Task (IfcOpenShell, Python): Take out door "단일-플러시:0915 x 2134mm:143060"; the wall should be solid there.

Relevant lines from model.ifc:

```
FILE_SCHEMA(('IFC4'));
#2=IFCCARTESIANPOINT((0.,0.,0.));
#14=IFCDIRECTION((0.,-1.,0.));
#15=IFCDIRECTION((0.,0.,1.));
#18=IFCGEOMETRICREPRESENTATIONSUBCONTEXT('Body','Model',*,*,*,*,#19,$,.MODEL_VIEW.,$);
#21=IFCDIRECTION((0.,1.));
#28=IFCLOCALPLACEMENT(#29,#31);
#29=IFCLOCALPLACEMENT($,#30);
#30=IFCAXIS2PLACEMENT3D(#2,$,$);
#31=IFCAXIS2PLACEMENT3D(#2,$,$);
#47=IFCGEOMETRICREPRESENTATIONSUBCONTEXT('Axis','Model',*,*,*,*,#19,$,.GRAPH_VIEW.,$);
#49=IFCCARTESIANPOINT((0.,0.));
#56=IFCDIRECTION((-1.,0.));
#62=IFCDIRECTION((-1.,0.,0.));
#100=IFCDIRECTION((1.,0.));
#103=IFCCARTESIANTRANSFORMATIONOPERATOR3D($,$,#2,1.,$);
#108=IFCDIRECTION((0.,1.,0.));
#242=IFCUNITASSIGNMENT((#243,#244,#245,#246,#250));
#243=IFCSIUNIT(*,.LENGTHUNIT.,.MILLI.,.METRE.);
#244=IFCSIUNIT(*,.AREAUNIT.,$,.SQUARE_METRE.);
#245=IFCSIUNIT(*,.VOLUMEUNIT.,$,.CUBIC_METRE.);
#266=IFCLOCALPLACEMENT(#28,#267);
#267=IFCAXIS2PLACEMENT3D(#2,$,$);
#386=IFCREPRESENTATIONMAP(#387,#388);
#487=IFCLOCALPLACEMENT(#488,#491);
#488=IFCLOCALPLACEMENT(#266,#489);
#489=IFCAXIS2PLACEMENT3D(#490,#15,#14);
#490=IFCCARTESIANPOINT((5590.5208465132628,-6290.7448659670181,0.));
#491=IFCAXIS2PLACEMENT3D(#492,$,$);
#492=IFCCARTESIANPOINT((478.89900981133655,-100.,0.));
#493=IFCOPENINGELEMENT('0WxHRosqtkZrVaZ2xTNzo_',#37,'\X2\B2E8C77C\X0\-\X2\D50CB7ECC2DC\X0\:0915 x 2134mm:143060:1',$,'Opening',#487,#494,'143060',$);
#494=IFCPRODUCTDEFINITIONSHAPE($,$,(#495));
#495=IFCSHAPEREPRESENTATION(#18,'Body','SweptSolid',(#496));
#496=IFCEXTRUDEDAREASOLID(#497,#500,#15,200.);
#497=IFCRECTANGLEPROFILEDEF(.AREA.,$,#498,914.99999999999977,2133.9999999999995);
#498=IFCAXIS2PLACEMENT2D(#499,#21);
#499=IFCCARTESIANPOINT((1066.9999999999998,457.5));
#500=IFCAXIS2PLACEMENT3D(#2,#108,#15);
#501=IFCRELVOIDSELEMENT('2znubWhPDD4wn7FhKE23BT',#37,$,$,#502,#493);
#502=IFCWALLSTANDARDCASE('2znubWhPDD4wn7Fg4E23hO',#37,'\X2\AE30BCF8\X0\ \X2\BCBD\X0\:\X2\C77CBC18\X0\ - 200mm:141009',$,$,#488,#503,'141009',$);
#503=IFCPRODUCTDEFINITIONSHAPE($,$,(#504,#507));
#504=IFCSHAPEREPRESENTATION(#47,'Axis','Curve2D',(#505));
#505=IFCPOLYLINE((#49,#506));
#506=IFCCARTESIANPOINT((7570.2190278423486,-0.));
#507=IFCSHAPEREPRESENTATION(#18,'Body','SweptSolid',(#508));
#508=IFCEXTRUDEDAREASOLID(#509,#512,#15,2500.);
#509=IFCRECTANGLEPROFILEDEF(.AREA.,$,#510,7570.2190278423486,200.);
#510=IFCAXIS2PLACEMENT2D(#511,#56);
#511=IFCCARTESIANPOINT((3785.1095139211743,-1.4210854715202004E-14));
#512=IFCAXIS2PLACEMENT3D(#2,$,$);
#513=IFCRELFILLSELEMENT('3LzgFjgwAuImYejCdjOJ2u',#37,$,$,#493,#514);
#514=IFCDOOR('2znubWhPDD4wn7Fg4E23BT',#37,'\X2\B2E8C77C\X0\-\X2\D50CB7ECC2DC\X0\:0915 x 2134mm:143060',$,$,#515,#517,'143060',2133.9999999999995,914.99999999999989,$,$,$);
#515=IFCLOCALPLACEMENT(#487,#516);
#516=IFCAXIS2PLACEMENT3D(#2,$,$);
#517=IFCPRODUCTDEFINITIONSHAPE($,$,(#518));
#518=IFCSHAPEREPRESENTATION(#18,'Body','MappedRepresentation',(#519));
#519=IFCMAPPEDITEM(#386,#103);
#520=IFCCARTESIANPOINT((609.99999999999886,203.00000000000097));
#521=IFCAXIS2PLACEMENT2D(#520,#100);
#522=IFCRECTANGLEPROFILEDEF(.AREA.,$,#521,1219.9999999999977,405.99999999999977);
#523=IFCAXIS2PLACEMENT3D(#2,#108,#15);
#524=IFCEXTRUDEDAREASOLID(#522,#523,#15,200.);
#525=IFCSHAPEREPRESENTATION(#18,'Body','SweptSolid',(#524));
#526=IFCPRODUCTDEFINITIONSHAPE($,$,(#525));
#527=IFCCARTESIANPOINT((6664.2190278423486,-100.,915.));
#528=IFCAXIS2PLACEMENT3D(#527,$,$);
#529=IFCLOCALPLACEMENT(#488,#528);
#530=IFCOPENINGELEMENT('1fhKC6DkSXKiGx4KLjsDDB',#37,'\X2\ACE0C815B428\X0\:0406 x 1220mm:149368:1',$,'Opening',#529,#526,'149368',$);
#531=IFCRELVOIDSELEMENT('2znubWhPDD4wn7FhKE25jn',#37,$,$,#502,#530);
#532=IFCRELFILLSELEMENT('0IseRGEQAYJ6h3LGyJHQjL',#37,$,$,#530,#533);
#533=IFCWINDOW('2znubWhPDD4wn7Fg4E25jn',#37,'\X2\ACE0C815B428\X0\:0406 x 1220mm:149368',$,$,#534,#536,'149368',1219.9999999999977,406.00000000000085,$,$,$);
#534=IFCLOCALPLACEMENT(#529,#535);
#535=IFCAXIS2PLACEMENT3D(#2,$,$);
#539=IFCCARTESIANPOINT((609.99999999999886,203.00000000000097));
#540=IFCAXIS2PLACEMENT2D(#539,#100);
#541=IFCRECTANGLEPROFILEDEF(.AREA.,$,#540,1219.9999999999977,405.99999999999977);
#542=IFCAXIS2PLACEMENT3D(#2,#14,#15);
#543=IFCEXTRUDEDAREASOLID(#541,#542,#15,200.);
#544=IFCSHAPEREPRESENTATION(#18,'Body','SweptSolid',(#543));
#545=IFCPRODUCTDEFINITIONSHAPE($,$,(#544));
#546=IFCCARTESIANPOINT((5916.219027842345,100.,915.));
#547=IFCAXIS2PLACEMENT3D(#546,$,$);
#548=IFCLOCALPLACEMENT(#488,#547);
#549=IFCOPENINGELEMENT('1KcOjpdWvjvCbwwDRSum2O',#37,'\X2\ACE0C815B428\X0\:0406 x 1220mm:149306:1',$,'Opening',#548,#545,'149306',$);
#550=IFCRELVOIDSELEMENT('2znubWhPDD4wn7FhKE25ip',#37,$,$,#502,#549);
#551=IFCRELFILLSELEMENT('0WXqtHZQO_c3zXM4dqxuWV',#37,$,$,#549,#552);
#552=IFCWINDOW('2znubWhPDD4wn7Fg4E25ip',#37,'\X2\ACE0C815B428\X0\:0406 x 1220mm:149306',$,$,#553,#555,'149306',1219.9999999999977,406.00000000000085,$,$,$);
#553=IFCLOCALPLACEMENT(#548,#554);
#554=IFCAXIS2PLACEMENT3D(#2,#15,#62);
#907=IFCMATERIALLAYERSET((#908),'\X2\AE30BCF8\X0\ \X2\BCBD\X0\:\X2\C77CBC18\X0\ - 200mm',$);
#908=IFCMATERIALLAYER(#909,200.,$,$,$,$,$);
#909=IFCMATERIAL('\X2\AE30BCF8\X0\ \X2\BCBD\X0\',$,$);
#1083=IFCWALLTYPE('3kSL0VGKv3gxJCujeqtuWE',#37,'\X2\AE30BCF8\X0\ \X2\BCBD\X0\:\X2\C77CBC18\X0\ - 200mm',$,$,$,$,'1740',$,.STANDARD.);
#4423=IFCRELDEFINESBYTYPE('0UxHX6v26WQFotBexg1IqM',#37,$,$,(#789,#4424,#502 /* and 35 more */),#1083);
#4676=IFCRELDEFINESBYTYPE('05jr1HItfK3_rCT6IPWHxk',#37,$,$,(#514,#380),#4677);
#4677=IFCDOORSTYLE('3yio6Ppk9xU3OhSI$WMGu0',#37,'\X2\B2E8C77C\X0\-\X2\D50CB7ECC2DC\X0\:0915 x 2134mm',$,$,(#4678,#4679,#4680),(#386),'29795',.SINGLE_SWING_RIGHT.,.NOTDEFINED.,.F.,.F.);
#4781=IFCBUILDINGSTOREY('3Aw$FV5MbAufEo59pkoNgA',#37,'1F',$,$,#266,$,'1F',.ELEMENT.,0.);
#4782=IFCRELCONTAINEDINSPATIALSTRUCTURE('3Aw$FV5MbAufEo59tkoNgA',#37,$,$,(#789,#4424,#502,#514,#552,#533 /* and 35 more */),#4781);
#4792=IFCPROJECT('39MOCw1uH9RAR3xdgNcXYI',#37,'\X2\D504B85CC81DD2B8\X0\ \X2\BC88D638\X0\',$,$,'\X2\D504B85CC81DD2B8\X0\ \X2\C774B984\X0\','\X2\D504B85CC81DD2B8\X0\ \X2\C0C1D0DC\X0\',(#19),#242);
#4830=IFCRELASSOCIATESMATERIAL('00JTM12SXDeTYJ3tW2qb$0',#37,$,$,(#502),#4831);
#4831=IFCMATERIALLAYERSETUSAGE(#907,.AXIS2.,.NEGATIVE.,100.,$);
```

```python
import ifcopenshell
import ifcopenshell.api.feature
import ifcopenshell.api.root
import ifcopenshell.geom
import ifcopenshell.util.shape

model = ifcopenshell.open("model.ifc")
settings = ifcopenshell.geom.settings()


def volume(element):
    """Net volume in cubic metres, openings subtracted."""
    shape = ifcopenshell.geom.create_shape(settings, element)
    return ifcopenshell.util.shape.get_volume(shape.geometry)


door = model.by_id(514)
opening = door.FillsVoids[0].RelatingOpeningElement
wall = opening.VoidsElements[0].RelatingBuildingElement
before = volume(wall)

ifcopenshell.api.root.remove_product(model, product=door)
ifcopenshell.api.feature.remove_feature(model, feature=opening)

after = volume(wall)

print(f"wall volume {before:.3f} -> {after:.3f} m3")

model.write("model_rev.ifc")
```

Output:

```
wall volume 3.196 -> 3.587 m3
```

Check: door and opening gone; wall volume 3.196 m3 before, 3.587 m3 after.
